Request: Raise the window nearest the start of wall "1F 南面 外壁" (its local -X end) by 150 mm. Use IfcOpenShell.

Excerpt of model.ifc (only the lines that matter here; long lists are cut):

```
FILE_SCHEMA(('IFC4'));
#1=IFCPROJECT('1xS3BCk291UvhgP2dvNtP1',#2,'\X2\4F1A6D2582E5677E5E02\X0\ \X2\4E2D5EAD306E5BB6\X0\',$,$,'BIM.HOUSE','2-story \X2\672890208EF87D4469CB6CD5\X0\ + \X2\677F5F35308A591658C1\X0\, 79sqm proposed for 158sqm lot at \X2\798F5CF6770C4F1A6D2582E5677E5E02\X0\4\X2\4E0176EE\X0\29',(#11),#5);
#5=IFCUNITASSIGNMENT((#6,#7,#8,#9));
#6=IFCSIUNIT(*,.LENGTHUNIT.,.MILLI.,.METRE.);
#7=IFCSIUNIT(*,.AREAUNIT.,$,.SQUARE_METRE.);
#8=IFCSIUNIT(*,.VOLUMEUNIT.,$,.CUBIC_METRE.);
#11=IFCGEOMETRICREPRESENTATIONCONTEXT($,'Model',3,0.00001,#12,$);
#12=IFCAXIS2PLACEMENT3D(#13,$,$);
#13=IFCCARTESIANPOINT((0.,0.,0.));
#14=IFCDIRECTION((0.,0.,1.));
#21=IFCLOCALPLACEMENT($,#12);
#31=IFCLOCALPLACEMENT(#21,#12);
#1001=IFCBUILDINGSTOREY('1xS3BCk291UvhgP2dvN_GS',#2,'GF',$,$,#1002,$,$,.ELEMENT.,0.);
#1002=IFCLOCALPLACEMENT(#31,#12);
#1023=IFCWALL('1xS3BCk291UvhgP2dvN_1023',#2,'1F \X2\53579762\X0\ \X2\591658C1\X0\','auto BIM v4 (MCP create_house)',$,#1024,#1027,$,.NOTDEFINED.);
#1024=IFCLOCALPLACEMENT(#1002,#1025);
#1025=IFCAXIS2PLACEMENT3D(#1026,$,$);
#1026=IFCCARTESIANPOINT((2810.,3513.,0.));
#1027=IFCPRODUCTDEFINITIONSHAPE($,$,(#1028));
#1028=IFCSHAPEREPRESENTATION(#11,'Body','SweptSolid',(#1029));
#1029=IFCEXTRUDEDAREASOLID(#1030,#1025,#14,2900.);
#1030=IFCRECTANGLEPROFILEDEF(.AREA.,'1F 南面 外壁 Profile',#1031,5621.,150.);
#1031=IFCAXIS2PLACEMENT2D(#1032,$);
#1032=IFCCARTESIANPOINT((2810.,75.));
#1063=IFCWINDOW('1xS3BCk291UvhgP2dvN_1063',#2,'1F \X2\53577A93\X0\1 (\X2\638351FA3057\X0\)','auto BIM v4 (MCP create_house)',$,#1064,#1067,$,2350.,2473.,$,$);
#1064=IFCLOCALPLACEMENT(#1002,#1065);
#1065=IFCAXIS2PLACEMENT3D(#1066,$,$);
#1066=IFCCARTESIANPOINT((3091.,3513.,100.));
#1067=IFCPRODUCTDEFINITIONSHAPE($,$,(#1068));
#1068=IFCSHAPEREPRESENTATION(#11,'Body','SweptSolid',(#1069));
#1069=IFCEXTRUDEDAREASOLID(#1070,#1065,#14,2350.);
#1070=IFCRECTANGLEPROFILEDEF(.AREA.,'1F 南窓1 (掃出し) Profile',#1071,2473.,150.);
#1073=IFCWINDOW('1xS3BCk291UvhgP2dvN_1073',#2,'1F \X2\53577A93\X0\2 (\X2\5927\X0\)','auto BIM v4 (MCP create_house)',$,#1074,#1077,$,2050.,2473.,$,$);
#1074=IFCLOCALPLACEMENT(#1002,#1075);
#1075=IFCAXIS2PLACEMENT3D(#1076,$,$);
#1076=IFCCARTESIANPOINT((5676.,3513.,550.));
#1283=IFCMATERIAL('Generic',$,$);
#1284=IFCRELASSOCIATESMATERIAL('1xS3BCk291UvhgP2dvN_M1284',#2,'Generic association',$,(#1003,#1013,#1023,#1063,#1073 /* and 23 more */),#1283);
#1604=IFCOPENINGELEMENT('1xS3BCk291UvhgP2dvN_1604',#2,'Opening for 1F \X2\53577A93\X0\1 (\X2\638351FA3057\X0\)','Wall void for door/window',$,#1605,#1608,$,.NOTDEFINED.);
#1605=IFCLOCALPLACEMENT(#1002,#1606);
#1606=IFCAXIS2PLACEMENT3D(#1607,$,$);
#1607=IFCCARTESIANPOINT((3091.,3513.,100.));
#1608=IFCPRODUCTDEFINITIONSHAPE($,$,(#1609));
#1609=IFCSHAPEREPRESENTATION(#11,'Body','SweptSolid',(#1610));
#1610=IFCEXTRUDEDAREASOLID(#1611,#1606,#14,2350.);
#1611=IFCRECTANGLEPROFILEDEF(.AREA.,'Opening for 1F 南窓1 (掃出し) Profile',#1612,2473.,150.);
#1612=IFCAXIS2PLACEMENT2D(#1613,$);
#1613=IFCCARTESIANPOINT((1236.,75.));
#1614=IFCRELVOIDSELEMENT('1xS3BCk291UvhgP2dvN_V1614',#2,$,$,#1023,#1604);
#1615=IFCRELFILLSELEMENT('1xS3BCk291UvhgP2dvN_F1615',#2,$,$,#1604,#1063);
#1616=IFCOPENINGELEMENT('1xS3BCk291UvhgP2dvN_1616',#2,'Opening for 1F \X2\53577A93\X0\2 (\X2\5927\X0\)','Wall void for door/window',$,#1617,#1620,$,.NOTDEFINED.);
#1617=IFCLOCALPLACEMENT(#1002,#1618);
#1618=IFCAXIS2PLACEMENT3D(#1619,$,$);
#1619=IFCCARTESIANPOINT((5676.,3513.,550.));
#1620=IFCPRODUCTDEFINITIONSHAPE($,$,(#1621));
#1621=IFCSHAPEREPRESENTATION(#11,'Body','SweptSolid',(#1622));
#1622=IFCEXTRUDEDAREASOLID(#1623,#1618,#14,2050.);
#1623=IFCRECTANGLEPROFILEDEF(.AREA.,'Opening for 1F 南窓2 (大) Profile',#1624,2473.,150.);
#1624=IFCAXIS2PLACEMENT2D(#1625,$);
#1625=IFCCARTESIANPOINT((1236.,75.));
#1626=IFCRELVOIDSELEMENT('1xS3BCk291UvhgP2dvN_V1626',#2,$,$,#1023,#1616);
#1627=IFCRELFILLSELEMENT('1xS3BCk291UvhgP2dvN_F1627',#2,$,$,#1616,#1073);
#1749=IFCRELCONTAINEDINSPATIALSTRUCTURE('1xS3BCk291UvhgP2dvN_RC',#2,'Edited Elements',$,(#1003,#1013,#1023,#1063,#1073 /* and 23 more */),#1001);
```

```python
import numpy as np
import ifcopenshell
import ifcopenshell.api.geometry
import ifcopenshell.util.placement
import ifcopenshell.util.unit

model = ifcopenshell.open("model.ifc")
unit_scale = ifcopenshell.util.unit.calculate_unit_scale(model)

window = model.by_guid("1xS3BCk291UvhgP2dvN_1063")
opening = window.FillsVoids[0].RelatingOpeningElement
dz = 0.15 / unit_scale

shift = np.array([0.0, 0.0, dz])
# The window is not placed relative to its opening, so move both.
for product in (opening, window):
    matrix = ifcopenshell.util.placement.get_local_placement(product.ObjectPlacement)
    matrix[:3, 3] += shift
    ifcopenshell.api.geometry.edit_object_placement(model, product=product, matrix=matrix, is_si=False)

print(f"moved by {dz * unit_scale:+.3f} m")

model.write("model_updated.ifc")
```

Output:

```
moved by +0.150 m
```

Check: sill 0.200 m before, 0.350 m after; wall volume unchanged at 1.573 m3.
